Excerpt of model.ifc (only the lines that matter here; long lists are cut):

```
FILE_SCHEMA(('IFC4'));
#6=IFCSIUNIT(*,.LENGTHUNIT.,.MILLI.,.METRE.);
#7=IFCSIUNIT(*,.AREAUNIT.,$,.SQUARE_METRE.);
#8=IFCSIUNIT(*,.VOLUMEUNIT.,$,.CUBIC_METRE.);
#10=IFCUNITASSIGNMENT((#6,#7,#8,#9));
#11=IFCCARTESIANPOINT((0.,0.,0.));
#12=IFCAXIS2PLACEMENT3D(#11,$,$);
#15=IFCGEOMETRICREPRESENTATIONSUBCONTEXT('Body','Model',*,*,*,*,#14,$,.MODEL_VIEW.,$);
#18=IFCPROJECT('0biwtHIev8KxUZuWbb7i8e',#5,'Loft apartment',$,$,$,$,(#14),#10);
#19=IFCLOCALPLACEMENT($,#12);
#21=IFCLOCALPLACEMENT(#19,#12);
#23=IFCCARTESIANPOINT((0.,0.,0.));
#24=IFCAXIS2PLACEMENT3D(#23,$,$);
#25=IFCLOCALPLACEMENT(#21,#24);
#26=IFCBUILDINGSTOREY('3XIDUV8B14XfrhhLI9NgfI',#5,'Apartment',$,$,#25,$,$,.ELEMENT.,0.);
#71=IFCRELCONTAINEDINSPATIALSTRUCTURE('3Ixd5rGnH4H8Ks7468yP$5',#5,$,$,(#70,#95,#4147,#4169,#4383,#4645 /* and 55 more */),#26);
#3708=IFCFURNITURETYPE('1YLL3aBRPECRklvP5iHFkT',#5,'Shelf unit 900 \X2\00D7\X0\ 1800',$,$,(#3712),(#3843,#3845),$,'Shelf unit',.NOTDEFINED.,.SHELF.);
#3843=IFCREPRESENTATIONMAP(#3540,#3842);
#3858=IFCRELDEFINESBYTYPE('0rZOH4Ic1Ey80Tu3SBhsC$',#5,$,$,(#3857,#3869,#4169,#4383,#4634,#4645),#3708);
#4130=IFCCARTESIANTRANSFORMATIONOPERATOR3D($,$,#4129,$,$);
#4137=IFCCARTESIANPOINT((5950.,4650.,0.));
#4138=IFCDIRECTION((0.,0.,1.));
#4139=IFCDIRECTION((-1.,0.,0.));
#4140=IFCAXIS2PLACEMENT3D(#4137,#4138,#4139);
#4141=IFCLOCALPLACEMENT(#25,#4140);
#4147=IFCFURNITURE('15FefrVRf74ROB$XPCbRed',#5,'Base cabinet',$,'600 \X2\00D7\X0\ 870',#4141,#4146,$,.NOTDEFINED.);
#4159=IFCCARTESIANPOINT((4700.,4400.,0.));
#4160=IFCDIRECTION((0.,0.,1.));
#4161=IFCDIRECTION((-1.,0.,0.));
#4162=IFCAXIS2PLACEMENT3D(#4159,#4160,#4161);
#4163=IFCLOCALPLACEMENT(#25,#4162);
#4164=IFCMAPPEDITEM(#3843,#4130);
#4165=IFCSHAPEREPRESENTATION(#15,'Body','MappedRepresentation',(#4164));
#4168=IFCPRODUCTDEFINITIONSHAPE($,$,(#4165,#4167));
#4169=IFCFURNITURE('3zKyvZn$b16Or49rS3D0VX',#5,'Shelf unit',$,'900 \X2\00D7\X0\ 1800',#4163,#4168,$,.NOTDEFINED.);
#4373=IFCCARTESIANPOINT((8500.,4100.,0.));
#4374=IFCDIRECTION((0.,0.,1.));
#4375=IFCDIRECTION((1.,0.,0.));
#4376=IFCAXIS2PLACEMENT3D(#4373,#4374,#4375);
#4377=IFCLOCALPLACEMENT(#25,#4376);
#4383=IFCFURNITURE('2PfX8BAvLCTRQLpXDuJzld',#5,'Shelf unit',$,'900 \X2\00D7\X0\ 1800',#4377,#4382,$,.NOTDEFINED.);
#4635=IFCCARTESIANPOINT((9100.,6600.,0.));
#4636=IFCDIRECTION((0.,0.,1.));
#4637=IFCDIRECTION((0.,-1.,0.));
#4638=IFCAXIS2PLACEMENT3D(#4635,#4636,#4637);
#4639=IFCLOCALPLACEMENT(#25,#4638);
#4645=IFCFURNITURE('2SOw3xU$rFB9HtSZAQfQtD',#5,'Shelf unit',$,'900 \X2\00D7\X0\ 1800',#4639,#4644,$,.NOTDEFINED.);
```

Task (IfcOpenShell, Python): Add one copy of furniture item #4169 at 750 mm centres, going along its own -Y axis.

```python
import ifcopenshell
import ifcopenshell.api.geometry
import ifcopenshell.api.root
import ifcopenshell.util.element
import ifcopenshell.util.placement
import ifcopenshell.util.unit

model = ifcopenshell.open("model.ifc")
unit_scale = ifcopenshell.util.unit.calculate_unit_scale(model)

source = model.by_guid("3zKyvZn$b16Or49rS3D0VX")
base = ifcopenshell.util.placement.get_local_placement(source.ObjectPlacement)
step = -base[:3, 1] * 0.75 / unit_scale

for i in range(1, 2):
    copy = ifcopenshell.api.root.copy_class(model, product=source)
    copy.Representation = ifcopenshell.util.element.copy_deep(
        model, source.Representation, exclude=["IfcGeometricRepresentationContext", "IfcRepresentationMap"]
    )
    matrix = base.copy()
    matrix[:3, 3] += i * step
    print("added at", matrix[:3, 3].round(3) + 0.0)
    ifcopenshell.api.geometry.edit_object_placement(model, product=copy, matrix=matrix, is_si=False)

model.write("model_updated.ifc")
```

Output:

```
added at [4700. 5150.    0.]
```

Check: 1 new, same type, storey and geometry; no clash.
